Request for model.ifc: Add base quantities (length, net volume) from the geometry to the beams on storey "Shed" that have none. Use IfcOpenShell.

First a look at what the model holds.

```python
import ifcopenshell
import ifcopenshell.util.element
import ifcopenshell.util.unit

model = ifcopenshell.open("model.ifc")
print(model.schema)
for unit_type in ("LENGTHUNIT", "AREAUNIT", "VOLUMEUNIT"):
    print(unit_type, ifcopenshell.util.unit.calculate_unit_scale(model, unit_type))
storey = next(s for s in model.by_type("IfcBuildingStorey") if s.Name == "Shed")
beams = [e for e in ifcopenshell.util.element.get_decomposition(storey) if e.is_a("IfcBeam")]
for e in sorted(beams, key=lambda e: e.id()):
    print(e.id(), e.is_a(), e.Name, list(ifcopenshell.util.element.get_psets(e, qtos_only=True)), sep=" | ")
```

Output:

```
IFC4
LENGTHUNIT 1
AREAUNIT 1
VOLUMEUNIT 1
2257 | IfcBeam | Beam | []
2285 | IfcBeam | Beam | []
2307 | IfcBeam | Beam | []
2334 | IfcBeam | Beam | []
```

```python
import ifcopenshell
import ifcopenshell.api.pset
import ifcopenshell.geom
import ifcopenshell.util.element
import ifcopenshell.util.shape
import ifcopenshell.util.unit

model = ifcopenshell.open("model.ifc")
unit_scale = ifcopenshell.util.unit.calculate_unit_scale(model)
volume_scale = ifcopenshell.util.unit.calculate_unit_scale(model, "VOLUMEUNIT")
settings = ifcopenshell.geom.settings()

storey = next(s for s in model.by_type("IfcBuildingStorey") if s.Name == "Shed")
beams = [e for e in ifcopenshell.util.element.get_decomposition(storey) if e.is_a("IfcBeam")]

for e in sorted(beams, key=lambda e: e.id()):
    if ifcopenshell.util.element.get_psets(e, qtos_only=True, should_inherit=False):
        continue
    # Geometry comes back in metres, in the element's own axes.
    shape = ifcopenshell.geom.create_shape(settings, e)
    values = {
        "Length": ifcopenshell.util.shape.get_max_xyz(shape.geometry) / unit_scale,
        "NetVolume": ifcopenshell.util.shape.get_volume(shape.geometry) / volume_scale,
    }
    qto = ifcopenshell.api.pset.add_qto(model, product=e, name="Qto_BeamBaseQuantities")
    ifcopenshell.api.pset.edit_qto(model, qto=qto, properties=values)
    print(e.id(), {k: round(v, 3) for k, v in values.items()})

model.write("model_edited.ifc")
```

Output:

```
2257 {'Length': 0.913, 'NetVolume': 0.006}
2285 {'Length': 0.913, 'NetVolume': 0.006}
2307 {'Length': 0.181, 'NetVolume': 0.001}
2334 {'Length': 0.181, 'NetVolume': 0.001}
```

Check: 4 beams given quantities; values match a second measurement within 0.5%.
